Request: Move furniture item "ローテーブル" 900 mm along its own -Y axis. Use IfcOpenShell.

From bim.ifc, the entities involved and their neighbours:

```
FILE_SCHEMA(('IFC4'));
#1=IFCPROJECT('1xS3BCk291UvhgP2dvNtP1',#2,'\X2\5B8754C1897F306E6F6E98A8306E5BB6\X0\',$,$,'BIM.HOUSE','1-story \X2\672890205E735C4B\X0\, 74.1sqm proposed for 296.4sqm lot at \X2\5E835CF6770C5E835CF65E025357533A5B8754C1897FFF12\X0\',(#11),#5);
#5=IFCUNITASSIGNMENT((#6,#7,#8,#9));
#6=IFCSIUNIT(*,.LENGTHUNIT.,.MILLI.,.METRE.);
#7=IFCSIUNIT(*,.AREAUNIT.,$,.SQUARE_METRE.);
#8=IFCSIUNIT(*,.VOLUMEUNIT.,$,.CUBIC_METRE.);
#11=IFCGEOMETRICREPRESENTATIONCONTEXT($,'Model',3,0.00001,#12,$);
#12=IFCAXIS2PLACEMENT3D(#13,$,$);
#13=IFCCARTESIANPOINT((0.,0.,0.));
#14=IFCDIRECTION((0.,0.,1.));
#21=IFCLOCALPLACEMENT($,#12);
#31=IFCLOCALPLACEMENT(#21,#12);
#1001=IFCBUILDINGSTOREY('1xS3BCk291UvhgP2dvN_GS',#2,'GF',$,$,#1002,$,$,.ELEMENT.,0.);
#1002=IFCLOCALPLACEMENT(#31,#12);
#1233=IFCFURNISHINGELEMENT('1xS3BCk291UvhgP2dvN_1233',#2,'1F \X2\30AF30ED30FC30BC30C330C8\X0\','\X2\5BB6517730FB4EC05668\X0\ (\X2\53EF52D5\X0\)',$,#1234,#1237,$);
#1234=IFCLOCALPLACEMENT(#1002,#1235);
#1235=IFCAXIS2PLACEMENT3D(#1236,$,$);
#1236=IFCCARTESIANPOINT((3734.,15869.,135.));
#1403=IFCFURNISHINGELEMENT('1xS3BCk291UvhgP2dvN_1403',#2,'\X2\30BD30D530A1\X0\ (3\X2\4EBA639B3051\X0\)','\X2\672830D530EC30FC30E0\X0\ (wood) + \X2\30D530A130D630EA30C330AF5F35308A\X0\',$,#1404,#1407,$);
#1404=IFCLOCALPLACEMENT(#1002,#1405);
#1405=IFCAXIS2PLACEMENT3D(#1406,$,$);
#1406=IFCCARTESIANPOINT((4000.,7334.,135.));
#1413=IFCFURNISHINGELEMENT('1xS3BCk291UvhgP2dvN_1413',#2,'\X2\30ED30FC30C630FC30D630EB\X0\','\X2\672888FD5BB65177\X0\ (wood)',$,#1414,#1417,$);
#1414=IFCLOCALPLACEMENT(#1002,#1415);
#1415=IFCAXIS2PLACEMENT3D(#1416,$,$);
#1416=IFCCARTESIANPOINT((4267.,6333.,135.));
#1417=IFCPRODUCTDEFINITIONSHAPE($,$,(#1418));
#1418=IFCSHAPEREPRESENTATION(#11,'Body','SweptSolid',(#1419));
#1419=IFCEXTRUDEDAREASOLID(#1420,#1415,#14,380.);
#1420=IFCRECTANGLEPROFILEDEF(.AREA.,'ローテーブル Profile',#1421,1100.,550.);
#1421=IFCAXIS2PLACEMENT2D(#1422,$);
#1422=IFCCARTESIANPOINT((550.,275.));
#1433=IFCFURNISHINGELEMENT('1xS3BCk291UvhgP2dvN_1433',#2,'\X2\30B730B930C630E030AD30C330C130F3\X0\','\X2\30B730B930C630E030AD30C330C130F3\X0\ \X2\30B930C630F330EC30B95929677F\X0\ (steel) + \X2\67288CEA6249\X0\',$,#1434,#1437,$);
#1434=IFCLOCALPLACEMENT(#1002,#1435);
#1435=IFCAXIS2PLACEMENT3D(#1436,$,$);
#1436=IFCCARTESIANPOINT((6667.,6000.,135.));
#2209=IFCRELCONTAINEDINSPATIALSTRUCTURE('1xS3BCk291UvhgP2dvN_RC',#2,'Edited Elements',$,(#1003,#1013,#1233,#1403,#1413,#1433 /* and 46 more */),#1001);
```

```python
import ifcopenshell
import ifcopenshell.api.geometry
import ifcopenshell.util.placement
import ifcopenshell.util.unit

model = ifcopenshell.open("bim.ifc")
unit_scale = ifcopenshell.util.unit.calculate_unit_scale(model)

item = model.by_guid("1xS3BCk291UvhgP2dvN_1413")
matrix = ifcopenshell.util.placement.get_local_placement(item.ObjectPlacement)
matrix[:3, 3] -= matrix[:3, 1] * 0.9 / unit_scale
ifcopenshell.api.geometry.edit_object_placement(model, product=item, matrix=matrix, is_si=False)

print(ifcopenshell.util.placement.get_local_placement(item.ObjectPlacement).round(3) + 0.0)

model.write("bim_rev.ifc")
```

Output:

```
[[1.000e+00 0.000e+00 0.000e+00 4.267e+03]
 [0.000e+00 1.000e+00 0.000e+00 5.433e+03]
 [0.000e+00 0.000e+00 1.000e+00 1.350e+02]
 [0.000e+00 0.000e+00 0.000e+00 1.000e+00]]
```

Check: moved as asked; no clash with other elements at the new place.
